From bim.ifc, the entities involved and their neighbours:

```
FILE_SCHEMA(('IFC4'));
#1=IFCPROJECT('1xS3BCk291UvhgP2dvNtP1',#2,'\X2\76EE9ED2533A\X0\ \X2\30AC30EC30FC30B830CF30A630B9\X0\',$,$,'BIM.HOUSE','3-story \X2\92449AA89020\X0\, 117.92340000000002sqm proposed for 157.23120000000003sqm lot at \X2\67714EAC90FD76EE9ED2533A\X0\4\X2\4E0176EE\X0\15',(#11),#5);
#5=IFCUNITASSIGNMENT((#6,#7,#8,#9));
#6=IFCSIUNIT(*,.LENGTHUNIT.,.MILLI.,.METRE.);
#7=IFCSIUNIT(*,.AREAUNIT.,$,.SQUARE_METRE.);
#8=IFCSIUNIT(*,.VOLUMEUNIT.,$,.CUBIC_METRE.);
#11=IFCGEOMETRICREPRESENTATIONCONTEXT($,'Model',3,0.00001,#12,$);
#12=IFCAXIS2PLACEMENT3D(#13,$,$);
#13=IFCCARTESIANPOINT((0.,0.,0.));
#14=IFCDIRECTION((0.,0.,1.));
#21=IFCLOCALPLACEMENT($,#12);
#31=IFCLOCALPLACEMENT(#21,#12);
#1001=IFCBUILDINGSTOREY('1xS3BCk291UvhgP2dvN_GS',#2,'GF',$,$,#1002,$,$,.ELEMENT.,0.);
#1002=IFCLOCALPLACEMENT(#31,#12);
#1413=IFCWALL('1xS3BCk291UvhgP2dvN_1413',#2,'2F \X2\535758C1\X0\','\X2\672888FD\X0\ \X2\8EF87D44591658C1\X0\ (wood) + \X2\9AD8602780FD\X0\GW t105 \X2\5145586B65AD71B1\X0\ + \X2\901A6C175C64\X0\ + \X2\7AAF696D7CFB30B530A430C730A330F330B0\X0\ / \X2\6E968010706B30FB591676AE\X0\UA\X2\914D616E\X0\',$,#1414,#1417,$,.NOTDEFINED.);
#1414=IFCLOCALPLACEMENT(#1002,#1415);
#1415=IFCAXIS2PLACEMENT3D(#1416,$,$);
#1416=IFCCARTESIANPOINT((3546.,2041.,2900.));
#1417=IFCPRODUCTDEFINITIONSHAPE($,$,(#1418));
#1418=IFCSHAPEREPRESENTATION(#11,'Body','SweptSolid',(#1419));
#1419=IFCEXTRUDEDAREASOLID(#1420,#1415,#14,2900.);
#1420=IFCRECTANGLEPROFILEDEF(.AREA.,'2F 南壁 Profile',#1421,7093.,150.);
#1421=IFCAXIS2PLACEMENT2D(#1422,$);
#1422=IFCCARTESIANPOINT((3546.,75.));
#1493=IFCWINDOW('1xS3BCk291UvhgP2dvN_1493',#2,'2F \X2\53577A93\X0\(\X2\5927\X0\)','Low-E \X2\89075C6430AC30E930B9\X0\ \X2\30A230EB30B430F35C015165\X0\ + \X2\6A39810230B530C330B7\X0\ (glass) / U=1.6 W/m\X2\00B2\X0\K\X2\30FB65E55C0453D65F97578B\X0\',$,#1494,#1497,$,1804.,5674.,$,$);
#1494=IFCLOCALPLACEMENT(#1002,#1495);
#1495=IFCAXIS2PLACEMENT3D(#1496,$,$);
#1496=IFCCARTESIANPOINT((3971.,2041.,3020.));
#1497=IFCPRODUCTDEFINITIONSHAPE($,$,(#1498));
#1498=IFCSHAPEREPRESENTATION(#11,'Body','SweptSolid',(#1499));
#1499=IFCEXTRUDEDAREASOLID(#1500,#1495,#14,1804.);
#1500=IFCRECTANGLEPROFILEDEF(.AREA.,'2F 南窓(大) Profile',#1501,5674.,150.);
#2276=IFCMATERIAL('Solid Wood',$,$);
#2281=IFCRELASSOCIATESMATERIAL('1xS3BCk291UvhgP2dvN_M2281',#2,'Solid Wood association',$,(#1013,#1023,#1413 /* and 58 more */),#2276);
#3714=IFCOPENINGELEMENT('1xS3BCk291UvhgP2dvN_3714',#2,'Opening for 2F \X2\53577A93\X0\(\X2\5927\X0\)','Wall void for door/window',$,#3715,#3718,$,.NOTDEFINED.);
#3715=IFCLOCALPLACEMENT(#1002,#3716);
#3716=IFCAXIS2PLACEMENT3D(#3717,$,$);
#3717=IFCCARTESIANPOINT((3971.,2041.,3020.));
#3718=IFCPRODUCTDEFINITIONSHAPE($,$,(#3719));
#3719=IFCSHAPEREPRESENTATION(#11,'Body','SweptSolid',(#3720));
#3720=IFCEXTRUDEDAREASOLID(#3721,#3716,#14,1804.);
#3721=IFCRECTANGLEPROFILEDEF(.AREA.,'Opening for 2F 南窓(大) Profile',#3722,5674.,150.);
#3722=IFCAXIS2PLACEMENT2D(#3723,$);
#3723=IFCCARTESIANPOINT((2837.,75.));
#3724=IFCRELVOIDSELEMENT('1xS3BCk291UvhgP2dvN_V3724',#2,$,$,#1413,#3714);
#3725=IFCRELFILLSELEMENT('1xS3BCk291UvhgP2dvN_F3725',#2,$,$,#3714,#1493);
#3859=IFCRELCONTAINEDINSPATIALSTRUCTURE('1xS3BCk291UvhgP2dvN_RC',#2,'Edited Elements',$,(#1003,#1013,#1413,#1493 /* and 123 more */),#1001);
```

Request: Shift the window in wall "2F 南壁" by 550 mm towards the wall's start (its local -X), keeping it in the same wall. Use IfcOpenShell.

```python
import ifcopenshell
import ifcopenshell.api.geometry
import ifcopenshell.util.placement
import ifcopenshell.util.unit

model = ifcopenshell.open("bim.ifc")
unit_scale = ifcopenshell.util.unit.calculate_unit_scale(model)

window = model.by_guid("1xS3BCk291UvhgP2dvN_1493")
opening = window.FillsVoids[0].RelatingOpeningElement
wall = opening.VoidsElements[0].RelatingBuildingElement

wall_matrix = ifcopenshell.util.placement.get_local_placement(wall.ObjectPlacement)
shift = wall_matrix[:3, 0] * -0.55 / unit_scale
before = ifcopenshell.util.placement.get_local_placement(window.ObjectPlacement)[:3, 3].copy()

# The window is not placed relative to its opening, so move both.
for product in (opening, window):
    matrix = ifcopenshell.util.placement.get_local_placement(product.ObjectPlacement)
    matrix[:3, 3] += shift
    ifcopenshell.api.geometry.edit_object_placement(model, product=product, matrix=matrix, is_si=False)

after = ifcopenshell.util.placement.get_local_placement(window.ObjectPlacement)[:3, 3]
print("window moved by", (after - before).round(3) + 0.0)

model.write("bim-out.ifc")
```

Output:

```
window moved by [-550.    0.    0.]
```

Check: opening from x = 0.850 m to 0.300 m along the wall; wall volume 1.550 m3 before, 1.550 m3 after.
